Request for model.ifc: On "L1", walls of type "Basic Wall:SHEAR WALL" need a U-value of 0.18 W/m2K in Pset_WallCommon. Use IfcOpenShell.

First a look at what the model holds.

```python
import ifcopenshell
import ifcopenshell.util.element

model = ifcopenshell.open("model.ifc")
print(model.schema)
storey = next(s for s in model.by_type("IfcBuildingStorey") if s.Name == "L1")
walls = [e for e in ifcopenshell.util.element.get_decomposition(storey) if e.is_a("IfcWall")]
seen = {}
for e in walls:
    element_type = ifcopenshell.util.element.get_type(e)
    key = (element_type.Name if element_type != e and element_type else None, ifcopenshell.util.element.get_pset(e, "Pset_WallCommon", "ThermalTransmittance"))
    seen[key] = seen.get(key, 0) + 1
for (name, value), count in sorted(seen.items(), key=str):
    print(count, "x", name, "|", value)
```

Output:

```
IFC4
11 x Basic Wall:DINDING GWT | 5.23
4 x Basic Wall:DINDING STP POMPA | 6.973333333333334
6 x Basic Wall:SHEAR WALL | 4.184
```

```python
import ifcopenshell
import ifcopenshell.api.pset
import ifcopenshell.util.element

model = ifcopenshell.open("model.ifc")

storey = next(s for s in model.by_type("IfcBuildingStorey") if s.Name == "L1")
walls = [e for e in ifcopenshell.util.element.get_decomposition(storey) if e.is_a("IfcWall")]

count = 0
for e in walls:
    element_type = ifcopenshell.util.element.get_type(e)
    if element_type in (None, e) or element_type.Name != "Basic Wall:SHEAR WALL":
        continue
    # add_pset returns the element's existing set when there is one.
    pset = ifcopenshell.api.pset.add_pset(model, product=e, name="Pset_WallCommon")
    ifcopenshell.api.pset.edit_pset(model, pset=pset, properties={"ThermalTransmittance": 0.18})
    count += 1

print(count, "walls updated")

model.write("model_v2.ifc")
```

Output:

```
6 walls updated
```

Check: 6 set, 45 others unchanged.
